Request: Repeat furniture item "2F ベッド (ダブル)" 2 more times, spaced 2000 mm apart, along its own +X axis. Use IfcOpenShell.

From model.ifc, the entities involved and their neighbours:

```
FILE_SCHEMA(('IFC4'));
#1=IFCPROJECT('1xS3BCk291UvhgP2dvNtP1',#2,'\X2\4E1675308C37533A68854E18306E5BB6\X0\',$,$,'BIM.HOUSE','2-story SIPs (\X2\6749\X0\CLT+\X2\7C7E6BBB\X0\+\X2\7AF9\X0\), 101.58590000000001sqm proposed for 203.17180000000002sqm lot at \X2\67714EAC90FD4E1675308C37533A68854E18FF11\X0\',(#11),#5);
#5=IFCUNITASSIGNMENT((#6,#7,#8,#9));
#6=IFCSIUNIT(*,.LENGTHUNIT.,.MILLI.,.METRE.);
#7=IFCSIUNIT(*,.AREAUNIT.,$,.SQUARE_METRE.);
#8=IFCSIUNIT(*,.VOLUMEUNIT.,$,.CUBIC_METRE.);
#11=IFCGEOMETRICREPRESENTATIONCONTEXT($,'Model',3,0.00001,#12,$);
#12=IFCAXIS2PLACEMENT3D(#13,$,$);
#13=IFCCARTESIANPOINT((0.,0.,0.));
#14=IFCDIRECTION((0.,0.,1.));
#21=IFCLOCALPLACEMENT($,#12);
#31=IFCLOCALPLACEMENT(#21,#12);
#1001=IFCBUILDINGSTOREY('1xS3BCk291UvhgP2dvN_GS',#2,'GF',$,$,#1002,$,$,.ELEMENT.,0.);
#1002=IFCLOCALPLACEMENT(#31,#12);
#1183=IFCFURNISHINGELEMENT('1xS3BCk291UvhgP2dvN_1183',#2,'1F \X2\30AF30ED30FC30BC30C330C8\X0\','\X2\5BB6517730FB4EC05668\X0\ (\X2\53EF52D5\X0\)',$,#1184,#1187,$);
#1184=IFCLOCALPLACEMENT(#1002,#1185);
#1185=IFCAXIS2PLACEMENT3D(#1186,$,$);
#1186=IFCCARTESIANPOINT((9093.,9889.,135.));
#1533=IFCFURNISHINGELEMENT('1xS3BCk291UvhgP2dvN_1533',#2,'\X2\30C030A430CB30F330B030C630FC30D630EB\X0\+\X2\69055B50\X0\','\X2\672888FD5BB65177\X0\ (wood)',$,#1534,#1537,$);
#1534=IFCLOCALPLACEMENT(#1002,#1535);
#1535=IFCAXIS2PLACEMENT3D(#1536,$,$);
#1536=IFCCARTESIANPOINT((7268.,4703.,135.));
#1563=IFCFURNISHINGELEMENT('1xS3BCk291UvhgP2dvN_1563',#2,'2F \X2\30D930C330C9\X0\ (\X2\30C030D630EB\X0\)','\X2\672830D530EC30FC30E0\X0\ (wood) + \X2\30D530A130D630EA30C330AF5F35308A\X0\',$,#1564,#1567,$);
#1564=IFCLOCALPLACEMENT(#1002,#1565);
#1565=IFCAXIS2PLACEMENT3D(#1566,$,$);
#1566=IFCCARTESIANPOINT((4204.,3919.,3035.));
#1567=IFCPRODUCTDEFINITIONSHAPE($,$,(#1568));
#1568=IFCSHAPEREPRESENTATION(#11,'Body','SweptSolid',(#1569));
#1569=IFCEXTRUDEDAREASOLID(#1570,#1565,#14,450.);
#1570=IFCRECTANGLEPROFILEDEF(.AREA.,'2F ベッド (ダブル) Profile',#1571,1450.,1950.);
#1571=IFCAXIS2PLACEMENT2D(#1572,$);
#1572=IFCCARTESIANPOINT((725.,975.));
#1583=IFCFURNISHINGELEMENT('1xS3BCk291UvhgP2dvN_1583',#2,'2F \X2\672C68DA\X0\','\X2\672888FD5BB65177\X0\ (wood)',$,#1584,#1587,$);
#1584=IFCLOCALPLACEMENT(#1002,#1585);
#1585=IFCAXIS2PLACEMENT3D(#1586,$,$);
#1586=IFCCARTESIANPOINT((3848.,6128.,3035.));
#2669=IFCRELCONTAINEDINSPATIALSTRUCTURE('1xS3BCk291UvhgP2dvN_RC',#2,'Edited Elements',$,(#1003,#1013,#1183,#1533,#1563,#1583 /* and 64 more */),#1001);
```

```python
import ifcopenshell
import ifcopenshell.api.geometry
import ifcopenshell.api.root
import ifcopenshell.util.element
import ifcopenshell.util.placement
import ifcopenshell.util.unit

model = ifcopenshell.open("model.ifc")
unit_scale = ifcopenshell.util.unit.calculate_unit_scale(model)


def reuse_history(source, copy):
    """copy_class also copies each property set's owner history, people and application; keep the originals."""
    for rel in copy.IsDefinedBy:
        if rel.is_a("IfcRelDefinesByProperties") and (history := rel.RelatingPropertyDefinition.OwnerHistory):
            rel.RelatingPropertyDefinition.OwnerHistory = source.OwnerHistory
            ifcopenshell.util.element.remove_deep2(model, history)


source = model.by_guid("1xS3BCk291UvhgP2dvN_1563")
base = ifcopenshell.util.placement.get_local_placement(source.ObjectPlacement)
step = base[:3, 0] * 2 / unit_scale

for i in range(1, 3):
    copy = ifcopenshell.api.root.copy_class(model, product=source)
    copy.Representation = ifcopenshell.util.element.copy_deep(
        model, source.Representation, exclude=["IfcGeometricRepresentationContext", "IfcRepresentationMap"]
    )
    reuse_history(source, copy)
    matrix = base.copy()
    matrix[:3, 3] += i * step
    print("added at", matrix[:3, 3].round(3) + 0.0)
    ifcopenshell.api.geometry.edit_object_placement(model, product=copy, matrix=matrix, is_si=False)

model.write("model_v2.ifc")
```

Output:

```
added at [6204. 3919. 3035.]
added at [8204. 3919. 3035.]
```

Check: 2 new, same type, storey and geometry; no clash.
